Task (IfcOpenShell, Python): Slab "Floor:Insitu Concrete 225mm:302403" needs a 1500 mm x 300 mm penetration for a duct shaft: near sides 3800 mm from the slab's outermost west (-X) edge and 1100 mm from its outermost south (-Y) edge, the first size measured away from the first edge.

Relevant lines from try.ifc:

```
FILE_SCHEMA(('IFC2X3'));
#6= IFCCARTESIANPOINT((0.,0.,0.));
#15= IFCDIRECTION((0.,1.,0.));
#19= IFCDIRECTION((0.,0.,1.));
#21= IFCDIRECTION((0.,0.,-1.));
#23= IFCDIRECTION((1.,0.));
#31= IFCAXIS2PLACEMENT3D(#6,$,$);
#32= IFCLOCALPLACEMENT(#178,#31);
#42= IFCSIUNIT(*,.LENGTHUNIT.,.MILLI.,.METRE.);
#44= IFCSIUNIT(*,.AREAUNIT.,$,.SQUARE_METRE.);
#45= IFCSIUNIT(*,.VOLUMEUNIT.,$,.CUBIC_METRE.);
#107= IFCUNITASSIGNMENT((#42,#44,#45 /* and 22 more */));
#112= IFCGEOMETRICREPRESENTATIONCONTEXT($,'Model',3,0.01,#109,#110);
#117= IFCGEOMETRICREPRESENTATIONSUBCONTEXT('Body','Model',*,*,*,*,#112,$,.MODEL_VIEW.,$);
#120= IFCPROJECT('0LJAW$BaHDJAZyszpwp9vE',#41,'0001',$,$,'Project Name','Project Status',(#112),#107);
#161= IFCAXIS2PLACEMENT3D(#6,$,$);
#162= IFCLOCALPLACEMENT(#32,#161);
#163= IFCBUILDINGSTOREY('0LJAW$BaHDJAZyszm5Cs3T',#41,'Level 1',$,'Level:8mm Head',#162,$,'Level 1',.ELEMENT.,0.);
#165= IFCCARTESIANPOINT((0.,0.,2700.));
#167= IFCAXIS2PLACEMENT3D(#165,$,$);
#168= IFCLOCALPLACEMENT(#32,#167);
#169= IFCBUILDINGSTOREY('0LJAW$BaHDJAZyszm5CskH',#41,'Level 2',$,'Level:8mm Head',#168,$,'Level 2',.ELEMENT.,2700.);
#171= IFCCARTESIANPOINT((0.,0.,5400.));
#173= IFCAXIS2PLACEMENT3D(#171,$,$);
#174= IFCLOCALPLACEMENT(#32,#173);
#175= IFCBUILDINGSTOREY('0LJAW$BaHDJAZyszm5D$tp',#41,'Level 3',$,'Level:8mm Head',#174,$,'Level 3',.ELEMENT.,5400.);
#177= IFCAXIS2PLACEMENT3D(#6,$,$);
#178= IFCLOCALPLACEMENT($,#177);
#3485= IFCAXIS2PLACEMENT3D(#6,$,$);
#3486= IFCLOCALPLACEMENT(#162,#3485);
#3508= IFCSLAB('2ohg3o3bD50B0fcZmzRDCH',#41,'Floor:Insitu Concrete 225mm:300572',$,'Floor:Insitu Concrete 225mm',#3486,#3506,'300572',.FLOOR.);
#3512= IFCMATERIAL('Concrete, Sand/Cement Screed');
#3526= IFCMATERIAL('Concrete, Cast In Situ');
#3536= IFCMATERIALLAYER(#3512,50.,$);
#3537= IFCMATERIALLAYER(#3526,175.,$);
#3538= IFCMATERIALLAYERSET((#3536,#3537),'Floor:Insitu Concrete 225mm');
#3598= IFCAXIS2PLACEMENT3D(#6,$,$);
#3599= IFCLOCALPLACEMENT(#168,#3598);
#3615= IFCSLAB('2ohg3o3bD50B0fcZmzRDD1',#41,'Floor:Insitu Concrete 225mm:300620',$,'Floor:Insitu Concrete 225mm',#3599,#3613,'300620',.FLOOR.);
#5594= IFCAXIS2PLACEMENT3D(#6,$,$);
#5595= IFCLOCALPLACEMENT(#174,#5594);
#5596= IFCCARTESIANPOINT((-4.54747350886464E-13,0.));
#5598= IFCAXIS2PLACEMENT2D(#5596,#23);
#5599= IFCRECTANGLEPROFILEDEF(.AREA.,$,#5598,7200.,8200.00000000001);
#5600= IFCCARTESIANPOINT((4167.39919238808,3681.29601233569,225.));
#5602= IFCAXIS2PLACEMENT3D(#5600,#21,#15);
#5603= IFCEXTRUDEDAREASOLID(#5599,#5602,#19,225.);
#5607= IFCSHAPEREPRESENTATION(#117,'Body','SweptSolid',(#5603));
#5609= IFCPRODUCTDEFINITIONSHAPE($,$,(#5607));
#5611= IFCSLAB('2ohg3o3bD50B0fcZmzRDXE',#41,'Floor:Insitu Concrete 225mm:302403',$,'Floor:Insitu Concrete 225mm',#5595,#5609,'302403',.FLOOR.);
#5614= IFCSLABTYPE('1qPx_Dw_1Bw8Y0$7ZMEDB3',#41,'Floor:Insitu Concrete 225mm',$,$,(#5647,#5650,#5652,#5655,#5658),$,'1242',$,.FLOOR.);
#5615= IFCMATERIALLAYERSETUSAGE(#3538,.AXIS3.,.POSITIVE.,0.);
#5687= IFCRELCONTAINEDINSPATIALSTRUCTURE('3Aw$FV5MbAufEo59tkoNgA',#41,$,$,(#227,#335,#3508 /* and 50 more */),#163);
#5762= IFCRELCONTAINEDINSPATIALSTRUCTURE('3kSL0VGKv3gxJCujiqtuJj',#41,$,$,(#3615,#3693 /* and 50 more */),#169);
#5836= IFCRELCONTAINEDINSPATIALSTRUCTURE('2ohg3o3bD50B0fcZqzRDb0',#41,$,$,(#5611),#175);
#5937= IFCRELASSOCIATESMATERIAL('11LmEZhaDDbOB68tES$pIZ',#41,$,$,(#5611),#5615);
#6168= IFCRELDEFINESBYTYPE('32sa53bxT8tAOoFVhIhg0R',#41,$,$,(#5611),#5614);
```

```python
import numpy as np
import ifcopenshell
import ifcopenshell.api.feature
import ifcopenshell.api.geometry
import ifcopenshell.api.root
import ifcopenshell.geom
import ifcopenshell.util.placement
import ifcopenshell.util.representation
import ifcopenshell.util.shape
import ifcopenshell.util.unit

model = ifcopenshell.open("try.ifc")
unit_scale = ifcopenshell.util.unit.calculate_unit_scale(model)
settings = ifcopenshell.geom.settings()


def volume(element):
    """Net volume in cubic metres, openings subtracted."""
    shape = ifcopenshell.geom.create_shape(settings, element)
    return ifcopenshell.util.shape.get_volume(shape.geometry)


slab = model.by_id(5611)
before = volume(slab)

# Extent in the slab's own axes, in metres. The edges named are its -X and -Y sides.
slab_shape = ifcopenshell.geom.create_shape(settings, slab)
vertices = ifcopenshell.util.shape.get_vertices(slab_shape.geometry)
x_min, y_min, bottom = vertices.min(axis=0)
top = vertices[:, 2].max()

opening = ifcopenshell.api.root.create_entity(model, ifc_class="IfcOpeningElement", name="Duct shaft opening")
context = ifcopenshell.util.representation.get_context(model, "Model", "Body", "MODEL_VIEW")
width, depth = 1.5, 0.3
outline = [(0.0, 0.0), (width, 0.0), (width, depth), (0.0, depth), (0.0, 0.0)]
# Overshoot both faces by 50 mm so the cut is clean.
shape = ifcopenshell.api.geometry.add_slab_representation(
    model, context=context, depth=top - bottom + 0.1, polyline=outline
)
ifcopenshell.api.geometry.assign_representation(model, product=opening, representation=shape)

matrix = ifcopenshell.util.placement.get_local_placement(slab.ObjectPlacement)
matrix[:, 3] = matrix @ np.append(np.array([x_min + 3.8, y_min + 1.1, bottom - 0.05]) / unit_scale, 1.0)
ifcopenshell.api.geometry.edit_object_placement(model, product=opening, matrix=matrix, is_si=False)
ifcopenshell.api.feature.add_feature(model, feature=opening, element=slab)

after = volume(slab)

print(f"slab volume {before:.3f} -> {after:.3f} m3")

model.write("try_updated.ifc")
```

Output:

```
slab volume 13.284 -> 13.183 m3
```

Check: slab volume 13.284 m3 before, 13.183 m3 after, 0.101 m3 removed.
